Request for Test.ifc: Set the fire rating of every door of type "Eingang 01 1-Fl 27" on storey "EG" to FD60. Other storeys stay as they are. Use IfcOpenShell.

First a look at what the model holds.

```python
import ifcopenshell
import ifcopenshell.util.element

model = ifcopenshell.open("Test.ifc")
print(model.schema)
storey = next(s for s in model.by_type("IfcBuildingStorey") if s.Name == "EG")
doors = [e for e in ifcopenshell.util.element.get_decomposition(storey) if e.is_a("IfcDoor")]
seen = {}
for e in doors:
    element_type = ifcopenshell.util.element.get_type(e)
    key = (element_type.Name if element_type != e and element_type else None, ifcopenshell.util.element.get_pset(e, "Pset_DoorCommon", "FireRating"))
    seen[key] = seen.get(key, 0) + 1
for (name, value), count in sorted(seen.items(), key=str):
    print(count, "x", name, "|", value)
```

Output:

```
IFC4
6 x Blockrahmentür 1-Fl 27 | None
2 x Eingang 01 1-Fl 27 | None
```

```python
import ifcopenshell
import ifcopenshell.api.pset
import ifcopenshell.util.element

model = ifcopenshell.open("Test.ifc")

storey = next(s for s in model.by_type("IfcBuildingStorey") if s.Name == "EG")
doors = [e for e in ifcopenshell.util.element.get_decomposition(storey) if e.is_a("IfcDoor")]

count = 0
for e in doors:
    element_type = ifcopenshell.util.element.get_type(e)
    if element_type in (None, e) or element_type.Name != "Eingang 01 1-Fl 27":
        continue
    # add_pset returns the element's existing set when there is one.
    pset = ifcopenshell.api.pset.add_pset(model, product=e, name="Pset_DoorCommon")
    ifcopenshell.api.pset.edit_pset(model, pset=pset, properties={"FireRating": "FD60"})
    count += 1

print(count, "doors updated")

model.write("Test-out.ifc")
```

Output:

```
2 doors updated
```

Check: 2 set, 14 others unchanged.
